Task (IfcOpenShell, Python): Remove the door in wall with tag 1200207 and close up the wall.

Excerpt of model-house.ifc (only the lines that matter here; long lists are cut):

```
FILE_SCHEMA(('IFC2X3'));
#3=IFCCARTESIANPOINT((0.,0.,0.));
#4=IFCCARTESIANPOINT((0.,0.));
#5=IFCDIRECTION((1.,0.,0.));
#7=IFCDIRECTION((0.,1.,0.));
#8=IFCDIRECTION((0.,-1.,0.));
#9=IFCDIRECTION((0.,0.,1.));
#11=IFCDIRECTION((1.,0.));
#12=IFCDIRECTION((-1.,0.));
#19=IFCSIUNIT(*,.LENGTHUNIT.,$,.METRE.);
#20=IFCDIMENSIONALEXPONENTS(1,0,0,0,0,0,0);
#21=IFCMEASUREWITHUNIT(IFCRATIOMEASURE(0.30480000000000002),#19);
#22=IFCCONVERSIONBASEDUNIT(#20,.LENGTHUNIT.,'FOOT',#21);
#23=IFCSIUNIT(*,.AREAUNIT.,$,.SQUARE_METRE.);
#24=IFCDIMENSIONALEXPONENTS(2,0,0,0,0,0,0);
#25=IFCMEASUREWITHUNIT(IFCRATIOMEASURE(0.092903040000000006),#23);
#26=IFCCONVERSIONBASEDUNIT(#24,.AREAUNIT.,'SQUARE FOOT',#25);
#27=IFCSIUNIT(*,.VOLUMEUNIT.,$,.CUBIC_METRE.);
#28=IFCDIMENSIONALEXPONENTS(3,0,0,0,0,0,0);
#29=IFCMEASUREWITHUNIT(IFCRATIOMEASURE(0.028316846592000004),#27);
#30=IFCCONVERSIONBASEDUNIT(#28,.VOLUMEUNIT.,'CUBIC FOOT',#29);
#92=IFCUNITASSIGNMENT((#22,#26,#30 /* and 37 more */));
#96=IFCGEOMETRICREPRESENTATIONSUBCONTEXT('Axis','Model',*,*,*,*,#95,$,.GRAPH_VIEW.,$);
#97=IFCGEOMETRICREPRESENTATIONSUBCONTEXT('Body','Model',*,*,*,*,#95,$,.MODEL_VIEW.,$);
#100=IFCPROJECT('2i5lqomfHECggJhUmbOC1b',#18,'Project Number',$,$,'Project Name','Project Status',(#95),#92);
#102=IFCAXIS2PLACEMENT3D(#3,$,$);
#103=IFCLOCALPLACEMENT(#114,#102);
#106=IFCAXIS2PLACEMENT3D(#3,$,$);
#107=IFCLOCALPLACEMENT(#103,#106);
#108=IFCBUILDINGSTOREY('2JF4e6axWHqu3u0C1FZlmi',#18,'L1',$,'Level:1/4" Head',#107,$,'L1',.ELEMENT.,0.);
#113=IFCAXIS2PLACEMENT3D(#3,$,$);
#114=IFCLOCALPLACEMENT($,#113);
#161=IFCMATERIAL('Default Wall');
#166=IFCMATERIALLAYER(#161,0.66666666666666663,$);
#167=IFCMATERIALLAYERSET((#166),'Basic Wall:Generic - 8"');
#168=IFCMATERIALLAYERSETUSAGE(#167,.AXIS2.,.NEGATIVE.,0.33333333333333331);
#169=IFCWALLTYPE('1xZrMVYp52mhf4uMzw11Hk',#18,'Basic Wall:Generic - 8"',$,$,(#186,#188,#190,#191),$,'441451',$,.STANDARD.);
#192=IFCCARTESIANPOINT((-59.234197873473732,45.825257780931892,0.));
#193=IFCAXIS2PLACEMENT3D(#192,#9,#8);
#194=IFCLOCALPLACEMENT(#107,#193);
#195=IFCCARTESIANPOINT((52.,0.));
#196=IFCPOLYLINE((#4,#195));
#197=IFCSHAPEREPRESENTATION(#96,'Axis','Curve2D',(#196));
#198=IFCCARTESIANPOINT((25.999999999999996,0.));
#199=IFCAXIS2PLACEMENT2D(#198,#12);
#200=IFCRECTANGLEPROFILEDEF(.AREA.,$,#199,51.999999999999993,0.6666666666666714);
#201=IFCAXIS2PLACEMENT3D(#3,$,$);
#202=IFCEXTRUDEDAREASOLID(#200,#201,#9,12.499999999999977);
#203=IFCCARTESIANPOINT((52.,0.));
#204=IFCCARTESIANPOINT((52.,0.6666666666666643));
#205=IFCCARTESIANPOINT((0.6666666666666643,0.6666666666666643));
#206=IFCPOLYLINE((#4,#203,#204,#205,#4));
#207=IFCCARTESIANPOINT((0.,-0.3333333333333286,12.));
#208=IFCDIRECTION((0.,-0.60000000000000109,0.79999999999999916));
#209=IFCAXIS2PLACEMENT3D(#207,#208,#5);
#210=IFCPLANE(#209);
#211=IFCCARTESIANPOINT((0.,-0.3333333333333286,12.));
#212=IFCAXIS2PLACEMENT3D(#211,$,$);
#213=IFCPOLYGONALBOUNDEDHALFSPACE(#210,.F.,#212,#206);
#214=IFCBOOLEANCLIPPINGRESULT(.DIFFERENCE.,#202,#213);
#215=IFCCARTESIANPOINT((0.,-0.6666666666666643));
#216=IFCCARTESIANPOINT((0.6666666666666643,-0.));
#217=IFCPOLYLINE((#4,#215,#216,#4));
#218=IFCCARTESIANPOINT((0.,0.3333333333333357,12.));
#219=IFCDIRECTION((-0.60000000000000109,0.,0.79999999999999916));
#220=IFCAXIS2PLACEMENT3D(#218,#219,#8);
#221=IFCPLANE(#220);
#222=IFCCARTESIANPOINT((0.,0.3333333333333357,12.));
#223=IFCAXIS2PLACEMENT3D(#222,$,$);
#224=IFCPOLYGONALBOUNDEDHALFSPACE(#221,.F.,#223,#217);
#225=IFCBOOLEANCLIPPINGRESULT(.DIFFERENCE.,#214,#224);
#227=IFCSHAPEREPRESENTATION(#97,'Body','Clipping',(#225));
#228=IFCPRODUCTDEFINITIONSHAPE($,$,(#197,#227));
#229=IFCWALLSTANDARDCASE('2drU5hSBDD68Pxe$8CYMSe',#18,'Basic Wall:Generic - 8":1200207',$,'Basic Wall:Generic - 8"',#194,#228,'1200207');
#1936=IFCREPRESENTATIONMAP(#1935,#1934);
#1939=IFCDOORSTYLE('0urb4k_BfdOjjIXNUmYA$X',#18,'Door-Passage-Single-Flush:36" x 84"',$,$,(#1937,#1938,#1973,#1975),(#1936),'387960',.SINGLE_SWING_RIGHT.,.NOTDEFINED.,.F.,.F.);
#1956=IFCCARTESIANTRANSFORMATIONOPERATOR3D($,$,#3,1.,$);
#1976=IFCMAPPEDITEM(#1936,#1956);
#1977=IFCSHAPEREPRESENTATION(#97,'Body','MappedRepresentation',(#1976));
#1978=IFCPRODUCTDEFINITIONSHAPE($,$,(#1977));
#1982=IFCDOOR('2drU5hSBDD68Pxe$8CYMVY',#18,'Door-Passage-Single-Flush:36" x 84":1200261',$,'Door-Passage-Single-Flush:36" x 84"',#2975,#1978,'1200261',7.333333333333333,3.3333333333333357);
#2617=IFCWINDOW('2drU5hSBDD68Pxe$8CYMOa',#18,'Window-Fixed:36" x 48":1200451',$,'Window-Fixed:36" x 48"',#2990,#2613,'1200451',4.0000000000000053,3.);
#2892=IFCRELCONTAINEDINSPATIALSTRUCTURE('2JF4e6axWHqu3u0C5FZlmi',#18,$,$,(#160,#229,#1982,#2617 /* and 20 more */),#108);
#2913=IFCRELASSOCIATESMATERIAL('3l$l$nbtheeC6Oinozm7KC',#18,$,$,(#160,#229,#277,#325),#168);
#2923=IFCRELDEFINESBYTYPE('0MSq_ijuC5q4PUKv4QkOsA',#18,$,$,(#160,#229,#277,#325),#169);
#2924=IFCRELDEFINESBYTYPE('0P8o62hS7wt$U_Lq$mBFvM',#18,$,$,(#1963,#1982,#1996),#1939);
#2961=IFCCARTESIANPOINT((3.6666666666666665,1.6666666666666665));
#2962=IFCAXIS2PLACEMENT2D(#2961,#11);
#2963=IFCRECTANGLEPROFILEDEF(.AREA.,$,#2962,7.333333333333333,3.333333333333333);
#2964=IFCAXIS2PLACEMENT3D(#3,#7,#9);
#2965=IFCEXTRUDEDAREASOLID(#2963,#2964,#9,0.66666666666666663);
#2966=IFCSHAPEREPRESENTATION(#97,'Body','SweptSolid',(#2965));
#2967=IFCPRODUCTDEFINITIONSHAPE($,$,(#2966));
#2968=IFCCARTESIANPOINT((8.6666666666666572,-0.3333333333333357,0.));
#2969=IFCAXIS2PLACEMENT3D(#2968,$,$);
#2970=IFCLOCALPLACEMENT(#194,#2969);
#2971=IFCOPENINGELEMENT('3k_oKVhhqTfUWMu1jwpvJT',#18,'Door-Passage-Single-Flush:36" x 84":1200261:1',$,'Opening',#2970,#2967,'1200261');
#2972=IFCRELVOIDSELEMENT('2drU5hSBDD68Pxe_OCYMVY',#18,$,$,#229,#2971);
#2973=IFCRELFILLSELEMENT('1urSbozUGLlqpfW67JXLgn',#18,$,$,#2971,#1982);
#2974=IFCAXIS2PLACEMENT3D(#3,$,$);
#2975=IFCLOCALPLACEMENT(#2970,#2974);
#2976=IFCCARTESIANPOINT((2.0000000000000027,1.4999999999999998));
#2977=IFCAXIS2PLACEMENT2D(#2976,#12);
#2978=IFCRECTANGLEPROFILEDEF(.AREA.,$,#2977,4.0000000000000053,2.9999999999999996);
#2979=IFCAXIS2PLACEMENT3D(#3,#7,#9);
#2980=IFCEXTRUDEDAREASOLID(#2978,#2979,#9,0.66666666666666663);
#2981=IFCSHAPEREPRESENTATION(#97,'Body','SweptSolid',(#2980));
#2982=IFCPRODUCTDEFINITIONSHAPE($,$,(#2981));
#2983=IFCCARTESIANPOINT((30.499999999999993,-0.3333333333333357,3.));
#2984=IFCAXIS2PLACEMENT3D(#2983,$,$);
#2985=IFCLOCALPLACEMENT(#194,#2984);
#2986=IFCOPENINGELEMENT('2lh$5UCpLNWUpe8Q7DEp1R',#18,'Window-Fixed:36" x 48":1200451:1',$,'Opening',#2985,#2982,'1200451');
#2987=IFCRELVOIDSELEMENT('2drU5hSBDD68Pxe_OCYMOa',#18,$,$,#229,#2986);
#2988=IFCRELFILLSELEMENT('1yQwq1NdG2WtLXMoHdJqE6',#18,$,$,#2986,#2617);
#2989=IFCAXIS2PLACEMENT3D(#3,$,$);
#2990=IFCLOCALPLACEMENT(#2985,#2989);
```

```python
import ifcopenshell
import ifcopenshell.api.feature
import ifcopenshell.api.root
import ifcopenshell.geom
import ifcopenshell.util.shape

model = ifcopenshell.open("model-house.ifc")
settings = ifcopenshell.geom.settings()


def volume(element):
    """Net volume in cubic metres, openings subtracted."""
    shape = ifcopenshell.geom.create_shape(settings, element)
    return ifcopenshell.util.shape.get_volume(shape.geometry)


door = model.by_guid("2drU5hSBDD68Pxe$8CYMVY")
opening = door.FillsVoids[0].RelatingOpeningElement
wall = opening.VoidsElements[0].RelatingBuildingElement
before = volume(wall)

ifcopenshell.api.root.remove_product(model, product=door)
ifcopenshell.api.feature.remove_feature(model, feature=opening)

after = volume(wall)

print(f"wall volume {before:.3f} -> {after:.3f} m3")

model.write("model-house_v2.ifc")
```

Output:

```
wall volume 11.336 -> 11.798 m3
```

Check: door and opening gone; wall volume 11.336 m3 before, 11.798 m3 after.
